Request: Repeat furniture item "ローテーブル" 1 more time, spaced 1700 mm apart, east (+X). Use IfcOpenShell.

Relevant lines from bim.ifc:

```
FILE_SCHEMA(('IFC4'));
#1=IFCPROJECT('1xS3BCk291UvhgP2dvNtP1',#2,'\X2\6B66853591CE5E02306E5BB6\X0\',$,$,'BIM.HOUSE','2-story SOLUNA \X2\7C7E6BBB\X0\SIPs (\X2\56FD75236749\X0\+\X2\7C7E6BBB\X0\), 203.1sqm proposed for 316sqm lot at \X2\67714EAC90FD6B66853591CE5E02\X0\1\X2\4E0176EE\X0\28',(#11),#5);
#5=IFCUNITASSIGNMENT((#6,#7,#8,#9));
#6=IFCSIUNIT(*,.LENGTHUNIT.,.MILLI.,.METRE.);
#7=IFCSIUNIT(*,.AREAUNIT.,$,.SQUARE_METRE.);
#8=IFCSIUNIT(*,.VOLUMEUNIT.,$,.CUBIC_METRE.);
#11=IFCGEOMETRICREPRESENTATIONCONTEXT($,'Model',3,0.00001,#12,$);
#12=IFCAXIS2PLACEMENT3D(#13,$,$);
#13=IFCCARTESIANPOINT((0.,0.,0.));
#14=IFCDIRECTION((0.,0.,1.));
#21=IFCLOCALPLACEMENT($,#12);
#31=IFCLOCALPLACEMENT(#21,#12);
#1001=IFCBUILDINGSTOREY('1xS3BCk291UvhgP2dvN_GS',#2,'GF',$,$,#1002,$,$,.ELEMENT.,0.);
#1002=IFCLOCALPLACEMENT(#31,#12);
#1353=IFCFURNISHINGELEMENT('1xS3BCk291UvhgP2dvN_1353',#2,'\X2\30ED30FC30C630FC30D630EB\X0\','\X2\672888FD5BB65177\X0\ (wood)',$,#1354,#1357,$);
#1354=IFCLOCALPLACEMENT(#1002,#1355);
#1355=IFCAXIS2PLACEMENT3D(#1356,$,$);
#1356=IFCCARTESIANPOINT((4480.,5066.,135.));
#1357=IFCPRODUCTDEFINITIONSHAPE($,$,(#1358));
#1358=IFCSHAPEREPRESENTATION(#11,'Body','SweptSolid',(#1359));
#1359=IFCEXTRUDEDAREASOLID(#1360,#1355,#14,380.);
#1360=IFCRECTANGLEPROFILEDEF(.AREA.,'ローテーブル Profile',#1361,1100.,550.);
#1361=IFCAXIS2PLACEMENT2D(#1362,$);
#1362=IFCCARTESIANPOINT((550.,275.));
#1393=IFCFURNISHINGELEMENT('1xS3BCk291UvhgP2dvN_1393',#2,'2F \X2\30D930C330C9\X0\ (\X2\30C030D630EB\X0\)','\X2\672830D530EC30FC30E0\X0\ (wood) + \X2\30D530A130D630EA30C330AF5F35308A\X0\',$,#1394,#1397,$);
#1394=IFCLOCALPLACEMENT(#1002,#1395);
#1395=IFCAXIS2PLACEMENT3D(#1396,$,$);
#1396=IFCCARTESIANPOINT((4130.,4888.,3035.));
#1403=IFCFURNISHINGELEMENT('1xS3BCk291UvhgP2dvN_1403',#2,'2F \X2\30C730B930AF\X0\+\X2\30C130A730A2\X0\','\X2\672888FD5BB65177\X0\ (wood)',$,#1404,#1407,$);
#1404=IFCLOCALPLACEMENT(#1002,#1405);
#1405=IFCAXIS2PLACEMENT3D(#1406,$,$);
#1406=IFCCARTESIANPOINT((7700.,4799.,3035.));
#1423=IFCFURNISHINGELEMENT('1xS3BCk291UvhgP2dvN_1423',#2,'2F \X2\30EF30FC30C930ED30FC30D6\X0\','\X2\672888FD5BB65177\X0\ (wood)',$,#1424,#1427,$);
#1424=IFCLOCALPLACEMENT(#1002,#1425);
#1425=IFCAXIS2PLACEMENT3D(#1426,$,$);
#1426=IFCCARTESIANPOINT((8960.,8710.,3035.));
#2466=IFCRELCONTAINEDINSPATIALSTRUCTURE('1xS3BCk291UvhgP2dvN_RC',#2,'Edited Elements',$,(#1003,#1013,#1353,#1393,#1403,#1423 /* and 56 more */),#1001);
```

```python
import numpy as np
import ifcopenshell
import ifcopenshell.api.geometry
import ifcopenshell.api.root
import ifcopenshell.util.element
import ifcopenshell.util.placement
import ifcopenshell.util.unit

model = ifcopenshell.open("bim.ifc")
unit_scale = ifcopenshell.util.unit.calculate_unit_scale(model)


def reuse_history(source, copy):
    """copy_class also copies each property set's owner history, people and application; keep the originals."""
    for rel in copy.IsDefinedBy:
        if rel.is_a("IfcRelDefinesByProperties") and (history := rel.RelatingPropertyDefinition.OwnerHistory):
            rel.RelatingPropertyDefinition.OwnerHistory = source.OwnerHistory
            ifcopenshell.util.element.remove_deep2(model, history)


source = model.by_guid("1xS3BCk291UvhgP2dvN_1353")
base = ifcopenshell.util.placement.get_local_placement(source.ObjectPlacement)
step = np.array([1.0, 0.0, 0.0]) * 1.7 / unit_scale

for i in range(1, 2):
    copy = ifcopenshell.api.root.copy_class(model, product=source)
    copy.Representation = ifcopenshell.util.element.copy_deep(
        model, source.Representation, exclude=["IfcGeometricRepresentationContext", "IfcRepresentationMap"]
    )
    reuse_history(source, copy)
    matrix = base.copy()
    matrix[:3, 3] += i * step
    print("added at", matrix[:3, 3].round(3) + 0.0)
    ifcopenshell.api.geometry.edit_object_placement(model, product=copy, matrix=matrix, is_si=False)

model.write("bim_edited.ifc")
```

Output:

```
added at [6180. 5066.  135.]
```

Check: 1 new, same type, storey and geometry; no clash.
